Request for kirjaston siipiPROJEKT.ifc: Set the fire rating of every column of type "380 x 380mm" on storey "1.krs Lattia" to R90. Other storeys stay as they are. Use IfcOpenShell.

First a look at what the model holds.

```python
import ifcopenshell
import ifcopenshell.util.element

model = ifcopenshell.open("kirjaston siipiPROJEKT.ifc")
print(model.schema)
storey = next(s for s in model.by_type("IfcBuildingStorey") if s.Name == "1.krs Lattia")
columns = [e for e in ifcopenshell.util.element.get_decomposition(storey) if e.is_a("IfcColumn")]
seen = {}
for e in columns:
    element_type = ifcopenshell.util.element.get_type(e)
    key = (element_type.Name if element_type != e and element_type else None, ifcopenshell.util.element.get_pset(e, "Pset_ColumnCommon", "FireRating"))
    seen[key] = seen.get(key, 0) + 1
for (name, value), count in sorted(seen.items(), key=str):
    print(count, "x", name, "|", value)
```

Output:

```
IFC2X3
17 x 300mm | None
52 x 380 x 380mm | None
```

```python
import ifcopenshell
import ifcopenshell.api.pset
import ifcopenshell.util.element

model = ifcopenshell.open("kirjaston siipiPROJEKT.ifc")

storey = next(s for s in model.by_type("IfcBuildingStorey") if s.Name == "1.krs Lattia")
columns = [e for e in ifcopenshell.util.element.get_decomposition(storey) if e.is_a("IfcColumn")]

count = 0
for e in columns:
    element_type = ifcopenshell.util.element.get_type(e)
    if element_type in (None, e) or element_type.Name != "380 x 380mm":
        continue
    # add_pset returns the element's existing set when there is one.
    pset = ifcopenshell.api.pset.add_pset(model, product=e, name="Pset_ColumnCommon")
    ifcopenshell.api.pset.edit_pset(model, pset=pset, properties={"FireRating": "R90"})
    count += 1

print(count, "columns updated")

model.write("kirjaston siipiPROJEKT_edited.ifc")
```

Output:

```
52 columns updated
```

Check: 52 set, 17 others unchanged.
